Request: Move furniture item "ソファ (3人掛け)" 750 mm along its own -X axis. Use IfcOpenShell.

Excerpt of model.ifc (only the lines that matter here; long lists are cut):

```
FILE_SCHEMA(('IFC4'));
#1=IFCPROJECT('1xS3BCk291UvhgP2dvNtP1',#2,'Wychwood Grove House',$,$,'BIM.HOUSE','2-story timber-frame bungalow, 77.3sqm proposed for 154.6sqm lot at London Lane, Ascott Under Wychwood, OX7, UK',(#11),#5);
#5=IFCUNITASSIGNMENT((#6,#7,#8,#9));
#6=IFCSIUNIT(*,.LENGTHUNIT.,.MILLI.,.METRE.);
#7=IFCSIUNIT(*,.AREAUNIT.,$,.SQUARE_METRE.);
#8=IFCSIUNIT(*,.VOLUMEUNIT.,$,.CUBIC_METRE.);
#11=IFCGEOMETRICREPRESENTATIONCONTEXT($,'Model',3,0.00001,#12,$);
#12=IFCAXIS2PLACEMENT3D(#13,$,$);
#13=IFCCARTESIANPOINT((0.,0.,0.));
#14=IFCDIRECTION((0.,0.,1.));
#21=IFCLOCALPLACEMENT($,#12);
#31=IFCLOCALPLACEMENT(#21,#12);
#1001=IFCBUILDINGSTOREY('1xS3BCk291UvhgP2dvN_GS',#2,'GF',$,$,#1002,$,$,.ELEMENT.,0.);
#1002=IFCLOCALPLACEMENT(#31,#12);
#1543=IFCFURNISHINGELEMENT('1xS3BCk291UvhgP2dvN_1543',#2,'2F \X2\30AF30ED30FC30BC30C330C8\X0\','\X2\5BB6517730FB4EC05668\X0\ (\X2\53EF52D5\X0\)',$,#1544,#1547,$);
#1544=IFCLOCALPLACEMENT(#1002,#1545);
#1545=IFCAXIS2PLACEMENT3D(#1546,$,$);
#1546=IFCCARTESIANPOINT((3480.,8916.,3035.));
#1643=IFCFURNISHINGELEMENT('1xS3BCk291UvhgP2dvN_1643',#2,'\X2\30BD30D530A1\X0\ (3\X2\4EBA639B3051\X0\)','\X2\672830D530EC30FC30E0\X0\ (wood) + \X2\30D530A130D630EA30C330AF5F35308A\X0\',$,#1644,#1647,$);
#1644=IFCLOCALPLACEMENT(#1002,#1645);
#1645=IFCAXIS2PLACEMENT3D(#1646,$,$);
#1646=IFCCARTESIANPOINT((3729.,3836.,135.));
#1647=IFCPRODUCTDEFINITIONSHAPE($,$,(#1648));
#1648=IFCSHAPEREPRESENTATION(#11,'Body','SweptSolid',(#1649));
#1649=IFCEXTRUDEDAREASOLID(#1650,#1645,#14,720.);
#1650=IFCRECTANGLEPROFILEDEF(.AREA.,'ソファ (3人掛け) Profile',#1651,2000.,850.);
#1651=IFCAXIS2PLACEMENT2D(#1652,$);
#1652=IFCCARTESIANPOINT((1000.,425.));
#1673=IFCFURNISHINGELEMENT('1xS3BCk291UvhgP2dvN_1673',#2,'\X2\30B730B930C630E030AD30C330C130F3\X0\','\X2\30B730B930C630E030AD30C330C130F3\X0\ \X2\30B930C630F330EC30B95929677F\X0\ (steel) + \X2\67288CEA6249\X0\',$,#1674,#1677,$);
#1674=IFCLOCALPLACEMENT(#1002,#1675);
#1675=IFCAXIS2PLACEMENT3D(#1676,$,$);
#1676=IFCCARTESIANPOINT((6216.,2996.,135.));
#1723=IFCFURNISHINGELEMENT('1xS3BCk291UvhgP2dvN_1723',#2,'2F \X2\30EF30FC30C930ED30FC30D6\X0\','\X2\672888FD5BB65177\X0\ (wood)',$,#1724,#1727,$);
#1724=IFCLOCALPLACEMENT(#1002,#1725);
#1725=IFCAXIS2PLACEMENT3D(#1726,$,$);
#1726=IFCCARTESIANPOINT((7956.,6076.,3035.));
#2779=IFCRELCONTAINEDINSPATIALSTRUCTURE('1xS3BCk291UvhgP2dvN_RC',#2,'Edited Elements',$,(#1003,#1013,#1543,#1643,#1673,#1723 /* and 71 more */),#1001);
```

```python
import ifcopenshell
import ifcopenshell.api.geometry
import ifcopenshell.util.placement
import ifcopenshell.util.unit

model = ifcopenshell.open("model.ifc")
unit_scale = ifcopenshell.util.unit.calculate_unit_scale(model)

item = model.by_id(1643)
matrix = ifcopenshell.util.placement.get_local_placement(item.ObjectPlacement)
matrix[:3, 3] -= matrix[:3, 0] * 0.75 / unit_scale
ifcopenshell.api.geometry.edit_object_placement(model, product=item, matrix=matrix, is_si=False)

print(ifcopenshell.util.placement.get_local_placement(item.ObjectPlacement).round(3) + 0.0)

model.write("model_v2.ifc")
```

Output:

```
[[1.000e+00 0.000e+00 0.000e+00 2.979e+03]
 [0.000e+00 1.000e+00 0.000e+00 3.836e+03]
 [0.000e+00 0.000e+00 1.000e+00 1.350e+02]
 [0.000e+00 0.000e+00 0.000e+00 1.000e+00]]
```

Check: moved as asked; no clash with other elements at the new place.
